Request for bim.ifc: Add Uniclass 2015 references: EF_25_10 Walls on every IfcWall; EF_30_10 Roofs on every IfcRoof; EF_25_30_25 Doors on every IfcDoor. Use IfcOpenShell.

First a look at what the model holds.

```python
import ifcopenshell

model = ifcopenshell.open("bim.ifc")
print(model.schema)
print("classifications:", [c.Name for c in model.by_type("IfcClassification")])
for ifc_class in ("IfcDoor", "IfcRoof", "IfcStair", "IfcWall", "IfcWindow"):
    print(ifc_class, len(model.by_type(ifc_class)))
```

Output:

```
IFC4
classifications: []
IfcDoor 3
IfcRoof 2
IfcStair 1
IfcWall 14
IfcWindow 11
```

```python
import ifcopenshell
import ifcopenshell.api.classification

model = ifcopenshell.open("bim.ifc")

system = ifcopenshell.api.classification.add_classification(model, classification="Uniclass 2015")

codes = {
    "IfcWall": ("EF_25_10", "Walls"),
    "IfcRoof": ("EF_30_10", "Roofs"),
    "IfcDoor": ("EF_25_30_25", "Doors"),
}
for ifc_class, (code, name) in codes.items():
    products = model.by_type(ifc_class)
    ifcopenshell.api.classification.add_reference(
        model, products=products, classification=system, identification=code, name=name
    )
    print(code, len(products))

model.write("bim_edited.ifc")
```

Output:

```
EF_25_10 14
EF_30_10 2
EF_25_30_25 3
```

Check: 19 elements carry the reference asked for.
